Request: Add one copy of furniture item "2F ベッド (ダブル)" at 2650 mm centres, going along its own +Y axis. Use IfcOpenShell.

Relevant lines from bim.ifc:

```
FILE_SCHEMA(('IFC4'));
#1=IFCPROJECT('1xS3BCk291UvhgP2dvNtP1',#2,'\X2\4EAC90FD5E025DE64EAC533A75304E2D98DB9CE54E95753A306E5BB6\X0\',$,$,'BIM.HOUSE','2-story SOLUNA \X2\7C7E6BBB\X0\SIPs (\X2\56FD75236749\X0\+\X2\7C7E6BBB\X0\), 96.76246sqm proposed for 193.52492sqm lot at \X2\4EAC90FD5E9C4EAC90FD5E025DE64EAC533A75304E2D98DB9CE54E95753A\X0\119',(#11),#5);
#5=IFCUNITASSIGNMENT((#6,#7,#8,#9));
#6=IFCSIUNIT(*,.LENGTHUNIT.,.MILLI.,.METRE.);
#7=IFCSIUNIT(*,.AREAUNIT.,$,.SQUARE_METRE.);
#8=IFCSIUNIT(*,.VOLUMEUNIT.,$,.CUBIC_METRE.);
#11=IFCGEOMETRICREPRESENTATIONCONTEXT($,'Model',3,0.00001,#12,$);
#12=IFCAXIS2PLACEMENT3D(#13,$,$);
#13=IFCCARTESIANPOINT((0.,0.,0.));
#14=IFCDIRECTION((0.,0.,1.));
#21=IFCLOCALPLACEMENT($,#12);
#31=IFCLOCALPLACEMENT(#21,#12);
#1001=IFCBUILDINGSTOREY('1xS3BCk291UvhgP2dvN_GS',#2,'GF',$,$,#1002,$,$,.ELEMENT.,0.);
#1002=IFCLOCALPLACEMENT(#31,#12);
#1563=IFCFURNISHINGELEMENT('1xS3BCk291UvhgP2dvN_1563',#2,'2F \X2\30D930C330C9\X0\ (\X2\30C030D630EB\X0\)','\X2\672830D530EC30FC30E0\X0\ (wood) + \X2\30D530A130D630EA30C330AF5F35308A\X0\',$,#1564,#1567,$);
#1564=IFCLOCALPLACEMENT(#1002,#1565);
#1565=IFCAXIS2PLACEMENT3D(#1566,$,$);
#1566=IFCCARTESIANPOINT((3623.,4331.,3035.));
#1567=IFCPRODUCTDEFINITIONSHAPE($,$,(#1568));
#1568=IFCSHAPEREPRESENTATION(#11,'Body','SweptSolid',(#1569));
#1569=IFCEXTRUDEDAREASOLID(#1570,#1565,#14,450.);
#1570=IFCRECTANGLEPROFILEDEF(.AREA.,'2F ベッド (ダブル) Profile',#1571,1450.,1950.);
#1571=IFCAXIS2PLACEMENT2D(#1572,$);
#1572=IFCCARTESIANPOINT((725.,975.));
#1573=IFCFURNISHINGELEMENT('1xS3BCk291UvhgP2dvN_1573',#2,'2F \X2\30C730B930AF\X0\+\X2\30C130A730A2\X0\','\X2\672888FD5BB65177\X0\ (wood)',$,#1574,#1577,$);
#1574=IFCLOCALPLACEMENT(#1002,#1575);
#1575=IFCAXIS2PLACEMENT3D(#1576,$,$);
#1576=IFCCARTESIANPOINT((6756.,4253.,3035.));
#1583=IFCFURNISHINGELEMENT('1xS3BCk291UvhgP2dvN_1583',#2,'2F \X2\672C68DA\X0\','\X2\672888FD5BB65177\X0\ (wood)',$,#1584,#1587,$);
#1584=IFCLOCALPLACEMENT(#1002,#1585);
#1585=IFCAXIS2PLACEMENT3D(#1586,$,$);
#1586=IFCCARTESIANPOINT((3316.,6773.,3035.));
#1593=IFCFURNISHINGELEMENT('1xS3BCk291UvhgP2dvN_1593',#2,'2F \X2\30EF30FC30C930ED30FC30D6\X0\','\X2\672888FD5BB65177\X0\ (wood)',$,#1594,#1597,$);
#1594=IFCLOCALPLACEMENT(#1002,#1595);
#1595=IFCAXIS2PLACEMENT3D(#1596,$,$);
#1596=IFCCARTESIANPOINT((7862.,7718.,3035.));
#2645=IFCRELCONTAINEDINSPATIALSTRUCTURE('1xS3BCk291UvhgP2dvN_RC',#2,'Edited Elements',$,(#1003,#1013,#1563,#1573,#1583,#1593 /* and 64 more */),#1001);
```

```python
import ifcopenshell
import ifcopenshell.api.geometry
import ifcopenshell.api.root
import ifcopenshell.util.element
import ifcopenshell.util.placement

model = ifcopenshell.open("bim.ifc")


def reuse_history(source, copy):
    """copy_class also copies each property set's owner history, people and application; keep the originals."""
    for rel in copy.IsDefinedBy:
        if rel.is_a("IfcRelDefinesByProperties") and (history := rel.RelatingPropertyDefinition.OwnerHistory):
            rel.RelatingPropertyDefinition.OwnerHistory = source.OwnerHistory
            ifcopenshell.util.element.remove_deep2(model, history)


source = model.by_id(1563)
base = ifcopenshell.util.placement.get_local_placement(source.ObjectPlacement)
step = base[:3, 1] * 2650.0

for i in range(1, 2):
    copy = ifcopenshell.api.root.copy_class(model, product=source)
    copy.Representation = ifcopenshell.util.element.copy_deep(
        model, source.Representation, exclude=["IfcGeometricRepresentationContext", "IfcRepresentationMap"]
    )
    reuse_history(source, copy)
    matrix = base.copy()
    matrix[:3, 3] += i * step
    print("added at", matrix[:3, 3].round(3) + 0.0)
    ifcopenshell.api.geometry.edit_object_placement(model, product=copy, matrix=matrix, is_si=False)

model.write("bim-out.ifc")
```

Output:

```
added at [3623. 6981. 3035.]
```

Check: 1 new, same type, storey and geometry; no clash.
